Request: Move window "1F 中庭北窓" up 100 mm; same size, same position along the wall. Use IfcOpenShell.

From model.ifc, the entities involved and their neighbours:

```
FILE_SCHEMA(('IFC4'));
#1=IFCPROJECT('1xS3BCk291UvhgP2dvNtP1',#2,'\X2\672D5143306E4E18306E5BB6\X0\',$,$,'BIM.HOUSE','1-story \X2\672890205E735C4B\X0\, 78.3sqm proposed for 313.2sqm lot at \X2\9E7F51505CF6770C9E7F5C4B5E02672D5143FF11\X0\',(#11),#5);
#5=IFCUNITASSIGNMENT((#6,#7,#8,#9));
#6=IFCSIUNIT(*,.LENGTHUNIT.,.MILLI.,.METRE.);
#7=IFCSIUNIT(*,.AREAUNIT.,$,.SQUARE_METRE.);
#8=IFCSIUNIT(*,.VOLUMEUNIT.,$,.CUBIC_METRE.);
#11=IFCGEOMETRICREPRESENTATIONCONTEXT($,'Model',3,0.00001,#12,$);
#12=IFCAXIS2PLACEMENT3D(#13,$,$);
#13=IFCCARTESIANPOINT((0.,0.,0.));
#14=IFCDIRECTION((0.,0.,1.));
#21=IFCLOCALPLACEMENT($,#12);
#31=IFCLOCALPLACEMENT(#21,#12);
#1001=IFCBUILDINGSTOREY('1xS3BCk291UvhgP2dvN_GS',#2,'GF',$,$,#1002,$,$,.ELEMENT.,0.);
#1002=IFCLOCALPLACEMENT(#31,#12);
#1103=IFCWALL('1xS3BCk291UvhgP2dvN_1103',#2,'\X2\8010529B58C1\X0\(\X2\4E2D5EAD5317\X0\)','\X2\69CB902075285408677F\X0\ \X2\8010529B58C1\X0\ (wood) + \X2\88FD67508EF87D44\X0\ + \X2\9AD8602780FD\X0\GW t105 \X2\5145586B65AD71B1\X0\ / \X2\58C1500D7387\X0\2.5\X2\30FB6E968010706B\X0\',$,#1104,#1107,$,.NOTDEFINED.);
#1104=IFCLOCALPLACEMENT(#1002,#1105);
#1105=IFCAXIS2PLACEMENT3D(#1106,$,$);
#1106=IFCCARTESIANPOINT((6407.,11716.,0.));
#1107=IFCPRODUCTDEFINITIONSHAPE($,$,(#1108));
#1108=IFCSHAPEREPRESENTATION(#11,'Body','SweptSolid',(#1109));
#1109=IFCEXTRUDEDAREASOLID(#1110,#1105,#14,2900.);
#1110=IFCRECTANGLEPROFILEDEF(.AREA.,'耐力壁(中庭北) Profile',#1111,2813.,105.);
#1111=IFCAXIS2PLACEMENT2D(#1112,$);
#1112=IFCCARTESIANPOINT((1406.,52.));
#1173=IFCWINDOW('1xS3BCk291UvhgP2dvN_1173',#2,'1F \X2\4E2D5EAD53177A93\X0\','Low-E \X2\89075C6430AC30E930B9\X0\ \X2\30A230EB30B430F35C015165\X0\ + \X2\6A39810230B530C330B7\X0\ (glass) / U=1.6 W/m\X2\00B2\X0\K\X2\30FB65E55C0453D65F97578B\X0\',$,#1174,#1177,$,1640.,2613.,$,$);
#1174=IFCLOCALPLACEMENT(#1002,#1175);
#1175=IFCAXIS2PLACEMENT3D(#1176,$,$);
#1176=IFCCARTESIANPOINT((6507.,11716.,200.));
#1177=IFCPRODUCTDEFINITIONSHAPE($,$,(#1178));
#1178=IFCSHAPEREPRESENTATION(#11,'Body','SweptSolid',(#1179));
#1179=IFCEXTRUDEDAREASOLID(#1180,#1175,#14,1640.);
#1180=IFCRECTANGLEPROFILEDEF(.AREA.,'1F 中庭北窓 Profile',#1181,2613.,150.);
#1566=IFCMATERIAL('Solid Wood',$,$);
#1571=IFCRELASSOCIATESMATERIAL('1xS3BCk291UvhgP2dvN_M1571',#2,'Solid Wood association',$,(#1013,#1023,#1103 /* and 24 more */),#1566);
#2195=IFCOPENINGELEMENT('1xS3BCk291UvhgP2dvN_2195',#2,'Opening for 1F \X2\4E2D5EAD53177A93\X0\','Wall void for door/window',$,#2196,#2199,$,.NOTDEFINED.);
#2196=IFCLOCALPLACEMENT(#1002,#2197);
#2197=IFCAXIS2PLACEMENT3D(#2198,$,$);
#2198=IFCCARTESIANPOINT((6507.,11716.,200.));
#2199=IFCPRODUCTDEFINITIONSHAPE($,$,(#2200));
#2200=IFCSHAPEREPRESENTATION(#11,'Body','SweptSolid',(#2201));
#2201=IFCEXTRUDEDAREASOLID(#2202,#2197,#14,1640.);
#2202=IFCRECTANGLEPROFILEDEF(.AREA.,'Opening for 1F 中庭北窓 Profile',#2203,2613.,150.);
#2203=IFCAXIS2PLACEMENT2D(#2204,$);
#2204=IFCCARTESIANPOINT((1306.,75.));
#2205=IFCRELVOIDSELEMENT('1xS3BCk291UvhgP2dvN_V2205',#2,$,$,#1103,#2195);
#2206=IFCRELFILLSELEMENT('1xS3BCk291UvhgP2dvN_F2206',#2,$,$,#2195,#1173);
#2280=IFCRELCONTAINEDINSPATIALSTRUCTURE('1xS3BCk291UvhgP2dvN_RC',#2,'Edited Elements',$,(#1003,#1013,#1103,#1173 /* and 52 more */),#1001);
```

```python
import numpy as np
import ifcopenshell
import ifcopenshell.api.geometry
import ifcopenshell.util.placement
import ifcopenshell.util.unit

model = ifcopenshell.open("model.ifc")
unit_scale = ifcopenshell.util.unit.calculate_unit_scale(model)

window = model.by_guid("1xS3BCk291UvhgP2dvN_1173")
opening = window.FillsVoids[0].RelatingOpeningElement
dz = 0.1 / unit_scale

shift = np.array([0.0, 0.0, dz])
# The window is not placed relative to its opening, so move both.
for product in (opening, window):
    matrix = ifcopenshell.util.placement.get_local_placement(product.ObjectPlacement)
    matrix[:3, 3] += shift
    ifcopenshell.api.geometry.edit_object_placement(model, product=product, matrix=matrix, is_si=False)

print(f"moved by {dz * unit_scale:+.3f} m")

model.write("model_rev.ifc")
```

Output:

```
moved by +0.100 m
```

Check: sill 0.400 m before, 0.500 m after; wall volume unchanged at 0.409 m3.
